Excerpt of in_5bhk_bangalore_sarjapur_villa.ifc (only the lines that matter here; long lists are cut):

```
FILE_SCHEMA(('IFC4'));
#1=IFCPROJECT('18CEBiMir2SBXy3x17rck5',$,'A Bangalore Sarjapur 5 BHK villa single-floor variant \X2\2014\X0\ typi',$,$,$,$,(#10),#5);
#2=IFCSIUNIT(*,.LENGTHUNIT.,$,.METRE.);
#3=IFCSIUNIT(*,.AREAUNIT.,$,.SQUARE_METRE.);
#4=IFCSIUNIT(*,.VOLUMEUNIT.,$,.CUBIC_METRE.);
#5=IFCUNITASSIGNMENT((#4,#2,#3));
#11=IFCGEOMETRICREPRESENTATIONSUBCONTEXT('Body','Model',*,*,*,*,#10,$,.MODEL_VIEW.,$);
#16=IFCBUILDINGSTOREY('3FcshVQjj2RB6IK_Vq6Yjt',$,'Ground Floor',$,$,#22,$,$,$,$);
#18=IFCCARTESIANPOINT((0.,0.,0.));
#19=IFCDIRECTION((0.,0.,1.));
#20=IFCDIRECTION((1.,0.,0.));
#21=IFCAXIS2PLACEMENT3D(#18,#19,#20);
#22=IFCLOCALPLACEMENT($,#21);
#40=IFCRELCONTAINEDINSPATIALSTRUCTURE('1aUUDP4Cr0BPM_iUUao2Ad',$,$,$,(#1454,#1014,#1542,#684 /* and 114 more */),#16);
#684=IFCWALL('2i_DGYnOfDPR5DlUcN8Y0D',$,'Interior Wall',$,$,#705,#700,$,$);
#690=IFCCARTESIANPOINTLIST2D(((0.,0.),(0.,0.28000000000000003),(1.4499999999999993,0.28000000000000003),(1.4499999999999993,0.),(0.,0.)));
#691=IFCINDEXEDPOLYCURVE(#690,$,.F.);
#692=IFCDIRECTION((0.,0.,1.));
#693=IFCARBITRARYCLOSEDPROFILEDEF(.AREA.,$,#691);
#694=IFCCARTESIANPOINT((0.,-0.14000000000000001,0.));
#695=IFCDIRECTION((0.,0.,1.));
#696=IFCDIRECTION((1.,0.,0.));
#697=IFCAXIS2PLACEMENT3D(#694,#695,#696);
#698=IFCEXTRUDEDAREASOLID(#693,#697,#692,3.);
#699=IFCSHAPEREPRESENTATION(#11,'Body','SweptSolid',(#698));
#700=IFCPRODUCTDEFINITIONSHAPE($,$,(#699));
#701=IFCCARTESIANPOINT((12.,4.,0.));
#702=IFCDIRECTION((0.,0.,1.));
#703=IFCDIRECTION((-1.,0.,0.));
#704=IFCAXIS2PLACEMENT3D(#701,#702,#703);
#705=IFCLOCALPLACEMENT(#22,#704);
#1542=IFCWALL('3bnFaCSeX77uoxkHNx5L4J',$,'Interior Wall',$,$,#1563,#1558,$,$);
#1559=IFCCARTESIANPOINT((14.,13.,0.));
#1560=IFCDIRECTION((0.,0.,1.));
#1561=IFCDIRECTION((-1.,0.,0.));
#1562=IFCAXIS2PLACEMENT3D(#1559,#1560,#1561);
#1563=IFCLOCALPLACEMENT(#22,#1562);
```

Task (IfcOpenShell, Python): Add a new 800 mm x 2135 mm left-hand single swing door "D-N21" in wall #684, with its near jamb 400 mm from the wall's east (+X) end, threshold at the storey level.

```python
import numpy as np
import ifcopenshell
import ifcopenshell.api.feature
import ifcopenshell.api.geometry
import ifcopenshell.api.root
import ifcopenshell.api.spatial
import ifcopenshell.geom
import ifcopenshell.util.element
import ifcopenshell.util.placement
import ifcopenshell.util.representation
import ifcopenshell.util.shape
import ifcopenshell.util.unit

model = ifcopenshell.open("in_5bhk_bangalore_sarjapur_villa.ifc")
unit_scale = ifcopenshell.util.unit.calculate_unit_scale(model)
settings = ifcopenshell.geom.settings()


def volume(element):
    """Net volume in cubic metres, openings subtracted."""
    shape = ifcopenshell.geom.create_shape(settings, element)
    return ifcopenshell.util.shape.get_volume(shape.geometry)


wall = model.by_guid("2i_DGYnOfDPR5DlUcN8Y0D")
storey = ifcopenshell.util.element.get_container(wall, ifc_class="IfcBuildingStorey")
context = ifcopenshell.util.representation.get_context(model, "Model", "Body", "MODEL_VIEW")
before = volume(wall)

width, height, from_end, sill = 0.8, 2.135, 0.4, 0.0  # metres

# The wall runs along its own X axis, and the end named is its -X end.
wall_shape = ifcopenshell.geom.create_shape(settings, wall)
x, y, z = ifcopenshell.util.shape.get_vertices(wall_shape.geometry).T
start = x.min() + from_end
face, thickness = float(y.min()), float(y.max() - y.min())
wall_matrix = ifcopenshell.util.placement.get_local_placement(wall.ObjectPlacement)
level = ifcopenshell.util.placement.get_local_placement(storey.ObjectPlacement)[2, 3]


def in_wall(x, y):
    """Placement at x, y metres in the wall's axes, at sill height."""
    matrix = wall_matrix.copy()
    matrix[:, 3] = wall_matrix @ np.array([x / unit_scale, y / unit_scale, 0.0, 1.0])
    matrix[2, 3] = level + sill / unit_scale
    return matrix


# Opening: a box that overshoots both wall faces by 50 mm.
opening = ifcopenshell.api.root.create_entity(model, ifc_class="IfcOpeningElement", predefined_type="OPENING")
box = ifcopenshell.api.geometry.add_wall_representation(
    model, context=context, length=width, height=height, thickness=thickness + 0.1
)
ifcopenshell.api.geometry.assign_representation(model, product=opening, representation=box)
ifcopenshell.api.geometry.edit_object_placement(model, product=opening, matrix=in_wall(start, face - 0.05), is_si=False)
ifcopenshell.api.feature.add_feature(model, feature=opening, element=wall)

door = ifcopenshell.api.root.create_entity(model, ifc_class="IfcDoor", name="D-N21", predefined_type="DOOR")
door.OverallWidth, door.OverallHeight = width / unit_scale, height / unit_scale
door.OperationType = "SINGLE_SWING_LEFT"
body = ifcopenshell.api.geometry.add_door_representation(
    model,
    context=context,
    overall_width=door.OverallWidth,
    overall_height=door.OverallHeight,
    operation_type="SINGLE_SWING_LEFT",
    lining_properties={"LiningDepth": thickness / unit_scale, "ThresholdDepth": thickness / unit_scale},
)
ifcopenshell.api.geometry.assign_representation(model, product=door, representation=body)
ifcopenshell.api.spatial.assign_container(model, products=[door], relating_structure=storey)
ifcopenshell.api.feature.add_filling(model, opening=opening, element=door)

# The lining spans the wall, so the door starts at the wall face.
ifcopenshell.api.geometry.edit_object_placement(model, product=door, matrix=in_wall(start, face), is_si=False)

after = volume(wall)

print(f"wall volume {before:.3f} -> {after:.3f} m3")

model.write("in_5bhk_bangalore_sarjapur_villa_rev.ifc")
```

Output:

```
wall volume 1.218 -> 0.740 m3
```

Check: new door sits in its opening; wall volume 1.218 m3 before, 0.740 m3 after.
